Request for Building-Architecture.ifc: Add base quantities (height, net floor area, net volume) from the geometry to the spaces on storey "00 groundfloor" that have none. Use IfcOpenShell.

First a look at what the model holds.

```python
import ifcopenshell
import ifcopenshell.util.element
import ifcopenshell.util.unit

model = ifcopenshell.open("Building-Architecture.ifc")
print(model.schema)
for unit_type in ("LENGTHUNIT", "AREAUNIT", "VOLUMEUNIT"):
    print(unit_type, ifcopenshell.util.unit.calculate_unit_scale(model, unit_type))
storey = next(s for s in model.by_type("IfcBuildingStorey") if s.Name == "00 groundfloor")
spaces = [e for e in ifcopenshell.util.element.get_decomposition(storey) if e.is_a("IfcSpace")]
for e in sorted(spaces, key=lambda e: e.id()):
    print(e.id(), e.is_a(), e.Name, list(ifcopenshell.util.element.get_psets(e, qtos_only=True)), sep=" | ")
```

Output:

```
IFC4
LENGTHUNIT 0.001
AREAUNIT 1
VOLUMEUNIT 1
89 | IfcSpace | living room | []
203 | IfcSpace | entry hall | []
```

```python
import ifcopenshell
import ifcopenshell.api.pset
import ifcopenshell.geom
import ifcopenshell.util.element
import ifcopenshell.util.shape
import ifcopenshell.util.unit

model = ifcopenshell.open("Building-Architecture.ifc")
unit_scale = ifcopenshell.util.unit.calculate_unit_scale(model)
area_scale = ifcopenshell.util.unit.calculate_unit_scale(model, "AREAUNIT")
volume_scale = ifcopenshell.util.unit.calculate_unit_scale(model, "VOLUMEUNIT")
settings = ifcopenshell.geom.settings()

storey = next(s for s in model.by_type("IfcBuildingStorey") if s.Name == "00 groundfloor")
spaces = [e for e in ifcopenshell.util.element.get_decomposition(storey) if e.is_a("IfcSpace")]

for e in sorted(spaces, key=lambda e: e.id()):
    if ifcopenshell.util.element.get_psets(e, qtos_only=True, should_inherit=False):
        continue
    # Geometry comes back in metres, in the element's own axes.
    shape = ifcopenshell.geom.create_shape(settings, e)
    values = {
        "Height": ifcopenshell.util.shape.get_z(shape.geometry) / unit_scale,
        "NetFloorArea": ifcopenshell.util.shape.get_footprint_area(shape.geometry) / area_scale,
        "NetVolume": ifcopenshell.util.shape.get_volume(shape.geometry) / volume_scale,
    }
    qto = ifcopenshell.api.pset.add_qto(model, product=e, name="Qto_SpaceBaseQuantities")
    ifcopenshell.api.pset.edit_qto(model, qto=qto, properties=values)
    print(e.id(), {k: round(v, 3) for k, v in values.items()})

model.write("Building-Architecture-out.ifc")
```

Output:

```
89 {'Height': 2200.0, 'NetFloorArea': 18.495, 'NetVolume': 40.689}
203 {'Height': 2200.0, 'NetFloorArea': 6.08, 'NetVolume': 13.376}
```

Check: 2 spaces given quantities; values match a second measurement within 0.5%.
